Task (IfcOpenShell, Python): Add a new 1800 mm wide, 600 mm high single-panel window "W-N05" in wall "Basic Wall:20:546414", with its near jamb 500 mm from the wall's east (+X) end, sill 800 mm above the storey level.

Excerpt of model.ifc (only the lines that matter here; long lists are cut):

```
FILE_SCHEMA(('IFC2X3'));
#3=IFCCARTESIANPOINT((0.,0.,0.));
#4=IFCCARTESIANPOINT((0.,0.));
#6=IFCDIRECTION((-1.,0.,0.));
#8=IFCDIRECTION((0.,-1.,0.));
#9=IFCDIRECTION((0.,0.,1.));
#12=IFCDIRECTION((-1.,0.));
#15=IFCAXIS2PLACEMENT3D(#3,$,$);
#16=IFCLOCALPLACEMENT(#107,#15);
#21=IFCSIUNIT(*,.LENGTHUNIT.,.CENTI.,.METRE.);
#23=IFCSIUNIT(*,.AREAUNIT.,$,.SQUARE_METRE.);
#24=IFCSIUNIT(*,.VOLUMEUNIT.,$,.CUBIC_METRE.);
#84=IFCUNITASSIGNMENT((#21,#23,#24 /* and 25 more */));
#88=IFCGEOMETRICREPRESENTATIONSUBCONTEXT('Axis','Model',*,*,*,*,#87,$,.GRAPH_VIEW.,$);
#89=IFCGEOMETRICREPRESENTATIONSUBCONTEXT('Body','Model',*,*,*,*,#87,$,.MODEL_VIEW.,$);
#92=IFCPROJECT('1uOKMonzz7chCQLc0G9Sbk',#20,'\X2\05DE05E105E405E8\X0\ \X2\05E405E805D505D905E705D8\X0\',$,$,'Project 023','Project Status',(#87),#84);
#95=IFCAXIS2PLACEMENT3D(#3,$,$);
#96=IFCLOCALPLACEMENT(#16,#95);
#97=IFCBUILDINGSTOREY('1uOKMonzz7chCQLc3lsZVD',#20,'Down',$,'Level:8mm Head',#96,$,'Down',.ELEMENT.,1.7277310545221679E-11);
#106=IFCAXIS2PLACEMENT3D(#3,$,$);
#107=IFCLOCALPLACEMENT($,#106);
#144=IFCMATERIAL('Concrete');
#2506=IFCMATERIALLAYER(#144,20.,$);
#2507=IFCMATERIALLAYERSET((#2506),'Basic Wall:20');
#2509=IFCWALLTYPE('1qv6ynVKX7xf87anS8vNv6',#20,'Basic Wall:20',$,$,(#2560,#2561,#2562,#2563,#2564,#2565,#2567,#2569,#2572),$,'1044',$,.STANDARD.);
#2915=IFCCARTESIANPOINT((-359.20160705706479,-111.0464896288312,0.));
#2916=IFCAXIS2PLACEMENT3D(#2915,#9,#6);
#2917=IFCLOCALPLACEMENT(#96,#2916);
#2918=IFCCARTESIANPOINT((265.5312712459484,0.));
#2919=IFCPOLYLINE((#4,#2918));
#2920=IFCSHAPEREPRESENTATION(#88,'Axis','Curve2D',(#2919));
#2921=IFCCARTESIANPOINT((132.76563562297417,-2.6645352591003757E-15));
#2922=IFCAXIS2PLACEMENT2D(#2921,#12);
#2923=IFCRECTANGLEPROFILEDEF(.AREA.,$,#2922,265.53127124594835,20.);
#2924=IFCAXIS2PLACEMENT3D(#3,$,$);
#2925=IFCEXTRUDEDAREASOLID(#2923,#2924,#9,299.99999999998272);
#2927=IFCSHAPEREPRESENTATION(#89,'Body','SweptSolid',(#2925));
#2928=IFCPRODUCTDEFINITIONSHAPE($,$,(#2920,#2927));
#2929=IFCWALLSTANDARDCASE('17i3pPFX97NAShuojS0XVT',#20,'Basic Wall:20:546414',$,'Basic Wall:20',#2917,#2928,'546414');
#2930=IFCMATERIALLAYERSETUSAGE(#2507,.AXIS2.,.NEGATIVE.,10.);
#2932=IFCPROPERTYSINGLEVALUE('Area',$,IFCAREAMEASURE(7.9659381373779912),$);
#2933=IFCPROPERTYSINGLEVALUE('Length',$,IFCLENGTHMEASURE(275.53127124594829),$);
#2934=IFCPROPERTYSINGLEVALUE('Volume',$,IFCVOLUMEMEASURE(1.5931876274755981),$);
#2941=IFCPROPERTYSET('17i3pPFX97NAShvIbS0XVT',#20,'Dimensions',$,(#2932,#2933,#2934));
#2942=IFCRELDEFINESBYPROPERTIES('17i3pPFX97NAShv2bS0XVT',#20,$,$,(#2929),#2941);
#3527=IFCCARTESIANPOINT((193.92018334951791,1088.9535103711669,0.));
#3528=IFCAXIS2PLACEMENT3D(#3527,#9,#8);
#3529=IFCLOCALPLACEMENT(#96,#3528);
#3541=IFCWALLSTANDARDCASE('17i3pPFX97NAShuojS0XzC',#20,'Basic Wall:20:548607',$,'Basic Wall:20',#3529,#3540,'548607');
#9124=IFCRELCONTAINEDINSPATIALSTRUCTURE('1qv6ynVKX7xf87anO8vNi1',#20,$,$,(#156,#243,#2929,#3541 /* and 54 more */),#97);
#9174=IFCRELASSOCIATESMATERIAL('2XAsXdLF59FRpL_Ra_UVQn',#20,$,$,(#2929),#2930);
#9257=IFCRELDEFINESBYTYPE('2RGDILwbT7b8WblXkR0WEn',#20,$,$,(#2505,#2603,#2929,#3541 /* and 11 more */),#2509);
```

```python
import numpy as np
import ifcopenshell
import ifcopenshell.api.feature
import ifcopenshell.api.geometry
import ifcopenshell.api.pset
import ifcopenshell.api.root
import ifcopenshell.api.spatial
import ifcopenshell.api.type
import ifcopenshell.geom
import ifcopenshell.util.element
import ifcopenshell.util.placement
import ifcopenshell.util.representation
import ifcopenshell.util.shape
import ifcopenshell.util.unit

model = ifcopenshell.open("model.ifc")
unit_scale = ifcopenshell.util.unit.calculate_unit_scale(model)
area_scale = ifcopenshell.util.unit.calculate_unit_scale(model, "AREAUNIT")
volume_scale = ifcopenshell.util.unit.calculate_unit_scale(model, "VOLUMEUNIT")
settings = ifcopenshell.geom.settings()


def volume(element):
    """Net volume in cubic metres, openings subtracted."""
    shape = ifcopenshell.geom.create_shape(settings, element)
    return ifcopenshell.util.shape.get_volume(shape.geometry)


wall = model.by_guid("17i3pPFX97NAShuojS0XVT")
storey = ifcopenshell.util.element.get_container(wall, ifc_class="IfcBuildingStorey")
context = ifcopenshell.util.representation.get_context(model, "Model", "Body", "MODEL_VIEW")
before = volume(wall)

width, height, from_end, sill = 1.8, 0.6, 0.5, 0.8  # metres

# The wall runs along its own X axis, and the end named is its -X end.
wall_shape = ifcopenshell.geom.create_shape(settings, wall)
x, y, z = ifcopenshell.util.shape.get_vertices(wall_shape.geometry).T
start = x.min() + from_end
face, thickness = float(y.min()), float(y.max() - y.min())
wall_matrix = ifcopenshell.util.placement.get_local_placement(wall.ObjectPlacement)
level = ifcopenshell.util.placement.get_local_placement(storey.ObjectPlacement)[2, 3]


def in_wall(x, y):
    """Placement at x, y metres in the wall's axes, at sill height."""
    matrix = wall_matrix.copy()
    matrix[:, 3] = wall_matrix @ np.array([x / unit_scale, y / unit_scale, 0.0, 1.0])
    matrix[2, 3] = level + sill / unit_scale
    return matrix


# Opening: a box that overshoots both wall faces by 50 mm.
opening = ifcopenshell.api.root.create_entity(model, ifc_class="IfcOpeningElement")
box = ifcopenshell.api.geometry.add_wall_representation(
    model, context=context, length=width, height=height, thickness=thickness + 0.1
)
ifcopenshell.api.geometry.assign_representation(model, product=opening, representation=box)
ifcopenshell.api.geometry.edit_object_placement(model, product=opening, matrix=in_wall(start, face - 0.05), is_si=False)
ifcopenshell.api.feature.add_feature(model, feature=opening, element=wall)

window = ifcopenshell.api.root.create_entity(model, ifc_class="IfcWindow", name="W-N05")
window.OverallWidth, window.OverallHeight = width / unit_scale, height / unit_scale
body = ifcopenshell.api.geometry.add_window_representation(
    model,
    context=context,
    overall_width=window.OverallWidth,
    overall_height=window.OverallHeight,
    partition_type="SINGLE_PANEL",
)
ifcopenshell.api.geometry.assign_representation(model, product=window, representation=body)
ifcopenshell.api.spatial.assign_container(model, products=[window], relating_structure=storey)
fills = ifcopenshell.api.feature.add_filling(model, opening=opening, element=window)
fills.OwnerHistory = window.OwnerHistory  # required in IFC2X3

# IFC2X3 keeps the operation on the window style.
style = ifcopenshell.api.root.create_entity(model, ifc_class="IfcWindowStyle", name="W-N05")
style.OperationType, style.ConstructionType = "SINGLE_PANEL", "NOTDEFINED"
style.ParameterTakesPrecedence = style.Sizeable = False
ifcopenshell.api.type.assign_type(model, related_objects=[window], relating_type=style)

# Centre the window in the wall's thickness.
ifcopenshell.api.geometry.edit_object_placement(model, product=window, matrix=in_wall(start, face), is_si=False)
window_shape = ifcopenshell.geom.create_shape(settings, window)
depth = ifcopenshell.util.shape.get_vertices(window_shape.geometry)[:, 1]
offset = face + thickness / 2 - (depth.min() + depth.max()) / 2
ifcopenshell.api.geometry.edit_object_placement(model, product=window, matrix=in_wall(start, offset), is_si=False)

after = volume(wall)

# Update the wall's stored quantities.
pset = model.by_id(ifcopenshell.util.element.get_pset(wall, "Dimensions", should_inherit=False)["id"])
ifcopenshell.api.pset.edit_pset(model, pset=pset, properties={
    "Area": model.create_entity("IfcAreaMeasure", after / thickness / area_scale),
    "Volume": model.create_entity("IfcVolumeMeasure", after / volume_scale),
})

print(f"wall volume {before:.3f} -> {after:.3f} m3")

model.write("model-out.ifc")
```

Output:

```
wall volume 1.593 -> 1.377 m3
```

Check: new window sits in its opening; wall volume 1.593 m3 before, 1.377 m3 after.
